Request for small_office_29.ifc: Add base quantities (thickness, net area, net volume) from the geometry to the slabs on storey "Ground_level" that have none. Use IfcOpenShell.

First a look at what the model holds.

```python
import ifcopenshell
import ifcopenshell.util.element
import ifcopenshell.util.unit

model = ifcopenshell.open("small_office_29.ifc")
print(model.schema)
for unit_type in ("LENGTHUNIT", "AREAUNIT", "VOLUMEUNIT"):
    print(unit_type, ifcopenshell.util.unit.calculate_unit_scale(model, unit_type))
storey = next(s for s in model.by_type("IfcBuildingStorey") if s.Name == "Ground_level")
slabs = [e for e in ifcopenshell.util.element.get_decomposition(storey) if e.is_a("IfcSlab")]
for e in sorted(slabs, key=lambda e: e.id()):
    print(e.id(), e.is_a(), e.Name, list(ifcopenshell.util.element.get_psets(e, qtos_only=True)), sep=" | ")
```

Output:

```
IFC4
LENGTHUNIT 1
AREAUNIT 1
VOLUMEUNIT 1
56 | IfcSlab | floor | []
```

```python
import ifcopenshell
import ifcopenshell.api.pset
import ifcopenshell.geom
import ifcopenshell.util.element
import ifcopenshell.util.shape
import ifcopenshell.util.unit

model = ifcopenshell.open("small_office_29.ifc")
unit_scale = ifcopenshell.util.unit.calculate_unit_scale(model)
area_scale = ifcopenshell.util.unit.calculate_unit_scale(model, "AREAUNIT")
volume_scale = ifcopenshell.util.unit.calculate_unit_scale(model, "VOLUMEUNIT")
settings = ifcopenshell.geom.settings()

storey = next(s for s in model.by_type("IfcBuildingStorey") if s.Name == "Ground_level")
slabs = [e for e in ifcopenshell.util.element.get_decomposition(storey) if e.is_a("IfcSlab")]

for e in sorted(slabs, key=lambda e: e.id()):
    if ifcopenshell.util.element.get_psets(e, qtos_only=True, should_inherit=False):
        continue
    # Geometry comes back in metres, in the element's own axes.
    shape = ifcopenshell.geom.create_shape(settings, e)
    values = {
        "Width": ifcopenshell.util.shape.get_z(shape.geometry) / unit_scale,
        "NetArea": ifcopenshell.util.shape.get_footprint_area(shape.geometry) / area_scale,
        "NetVolume": ifcopenshell.util.shape.get_volume(shape.geometry) / volume_scale,
    }
    qto = ifcopenshell.api.pset.add_qto(model, product=e, name="Qto_SlabBaseQuantities")
    ifcopenshell.api.pset.edit_qto(model, qto=qto, properties=values)
    print(e.id(), {k: round(v, 3) for k, v in values.items()})

model.write("small_office_29_updated.ifc")
```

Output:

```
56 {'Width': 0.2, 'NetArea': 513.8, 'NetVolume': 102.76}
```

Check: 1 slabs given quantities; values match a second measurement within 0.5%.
